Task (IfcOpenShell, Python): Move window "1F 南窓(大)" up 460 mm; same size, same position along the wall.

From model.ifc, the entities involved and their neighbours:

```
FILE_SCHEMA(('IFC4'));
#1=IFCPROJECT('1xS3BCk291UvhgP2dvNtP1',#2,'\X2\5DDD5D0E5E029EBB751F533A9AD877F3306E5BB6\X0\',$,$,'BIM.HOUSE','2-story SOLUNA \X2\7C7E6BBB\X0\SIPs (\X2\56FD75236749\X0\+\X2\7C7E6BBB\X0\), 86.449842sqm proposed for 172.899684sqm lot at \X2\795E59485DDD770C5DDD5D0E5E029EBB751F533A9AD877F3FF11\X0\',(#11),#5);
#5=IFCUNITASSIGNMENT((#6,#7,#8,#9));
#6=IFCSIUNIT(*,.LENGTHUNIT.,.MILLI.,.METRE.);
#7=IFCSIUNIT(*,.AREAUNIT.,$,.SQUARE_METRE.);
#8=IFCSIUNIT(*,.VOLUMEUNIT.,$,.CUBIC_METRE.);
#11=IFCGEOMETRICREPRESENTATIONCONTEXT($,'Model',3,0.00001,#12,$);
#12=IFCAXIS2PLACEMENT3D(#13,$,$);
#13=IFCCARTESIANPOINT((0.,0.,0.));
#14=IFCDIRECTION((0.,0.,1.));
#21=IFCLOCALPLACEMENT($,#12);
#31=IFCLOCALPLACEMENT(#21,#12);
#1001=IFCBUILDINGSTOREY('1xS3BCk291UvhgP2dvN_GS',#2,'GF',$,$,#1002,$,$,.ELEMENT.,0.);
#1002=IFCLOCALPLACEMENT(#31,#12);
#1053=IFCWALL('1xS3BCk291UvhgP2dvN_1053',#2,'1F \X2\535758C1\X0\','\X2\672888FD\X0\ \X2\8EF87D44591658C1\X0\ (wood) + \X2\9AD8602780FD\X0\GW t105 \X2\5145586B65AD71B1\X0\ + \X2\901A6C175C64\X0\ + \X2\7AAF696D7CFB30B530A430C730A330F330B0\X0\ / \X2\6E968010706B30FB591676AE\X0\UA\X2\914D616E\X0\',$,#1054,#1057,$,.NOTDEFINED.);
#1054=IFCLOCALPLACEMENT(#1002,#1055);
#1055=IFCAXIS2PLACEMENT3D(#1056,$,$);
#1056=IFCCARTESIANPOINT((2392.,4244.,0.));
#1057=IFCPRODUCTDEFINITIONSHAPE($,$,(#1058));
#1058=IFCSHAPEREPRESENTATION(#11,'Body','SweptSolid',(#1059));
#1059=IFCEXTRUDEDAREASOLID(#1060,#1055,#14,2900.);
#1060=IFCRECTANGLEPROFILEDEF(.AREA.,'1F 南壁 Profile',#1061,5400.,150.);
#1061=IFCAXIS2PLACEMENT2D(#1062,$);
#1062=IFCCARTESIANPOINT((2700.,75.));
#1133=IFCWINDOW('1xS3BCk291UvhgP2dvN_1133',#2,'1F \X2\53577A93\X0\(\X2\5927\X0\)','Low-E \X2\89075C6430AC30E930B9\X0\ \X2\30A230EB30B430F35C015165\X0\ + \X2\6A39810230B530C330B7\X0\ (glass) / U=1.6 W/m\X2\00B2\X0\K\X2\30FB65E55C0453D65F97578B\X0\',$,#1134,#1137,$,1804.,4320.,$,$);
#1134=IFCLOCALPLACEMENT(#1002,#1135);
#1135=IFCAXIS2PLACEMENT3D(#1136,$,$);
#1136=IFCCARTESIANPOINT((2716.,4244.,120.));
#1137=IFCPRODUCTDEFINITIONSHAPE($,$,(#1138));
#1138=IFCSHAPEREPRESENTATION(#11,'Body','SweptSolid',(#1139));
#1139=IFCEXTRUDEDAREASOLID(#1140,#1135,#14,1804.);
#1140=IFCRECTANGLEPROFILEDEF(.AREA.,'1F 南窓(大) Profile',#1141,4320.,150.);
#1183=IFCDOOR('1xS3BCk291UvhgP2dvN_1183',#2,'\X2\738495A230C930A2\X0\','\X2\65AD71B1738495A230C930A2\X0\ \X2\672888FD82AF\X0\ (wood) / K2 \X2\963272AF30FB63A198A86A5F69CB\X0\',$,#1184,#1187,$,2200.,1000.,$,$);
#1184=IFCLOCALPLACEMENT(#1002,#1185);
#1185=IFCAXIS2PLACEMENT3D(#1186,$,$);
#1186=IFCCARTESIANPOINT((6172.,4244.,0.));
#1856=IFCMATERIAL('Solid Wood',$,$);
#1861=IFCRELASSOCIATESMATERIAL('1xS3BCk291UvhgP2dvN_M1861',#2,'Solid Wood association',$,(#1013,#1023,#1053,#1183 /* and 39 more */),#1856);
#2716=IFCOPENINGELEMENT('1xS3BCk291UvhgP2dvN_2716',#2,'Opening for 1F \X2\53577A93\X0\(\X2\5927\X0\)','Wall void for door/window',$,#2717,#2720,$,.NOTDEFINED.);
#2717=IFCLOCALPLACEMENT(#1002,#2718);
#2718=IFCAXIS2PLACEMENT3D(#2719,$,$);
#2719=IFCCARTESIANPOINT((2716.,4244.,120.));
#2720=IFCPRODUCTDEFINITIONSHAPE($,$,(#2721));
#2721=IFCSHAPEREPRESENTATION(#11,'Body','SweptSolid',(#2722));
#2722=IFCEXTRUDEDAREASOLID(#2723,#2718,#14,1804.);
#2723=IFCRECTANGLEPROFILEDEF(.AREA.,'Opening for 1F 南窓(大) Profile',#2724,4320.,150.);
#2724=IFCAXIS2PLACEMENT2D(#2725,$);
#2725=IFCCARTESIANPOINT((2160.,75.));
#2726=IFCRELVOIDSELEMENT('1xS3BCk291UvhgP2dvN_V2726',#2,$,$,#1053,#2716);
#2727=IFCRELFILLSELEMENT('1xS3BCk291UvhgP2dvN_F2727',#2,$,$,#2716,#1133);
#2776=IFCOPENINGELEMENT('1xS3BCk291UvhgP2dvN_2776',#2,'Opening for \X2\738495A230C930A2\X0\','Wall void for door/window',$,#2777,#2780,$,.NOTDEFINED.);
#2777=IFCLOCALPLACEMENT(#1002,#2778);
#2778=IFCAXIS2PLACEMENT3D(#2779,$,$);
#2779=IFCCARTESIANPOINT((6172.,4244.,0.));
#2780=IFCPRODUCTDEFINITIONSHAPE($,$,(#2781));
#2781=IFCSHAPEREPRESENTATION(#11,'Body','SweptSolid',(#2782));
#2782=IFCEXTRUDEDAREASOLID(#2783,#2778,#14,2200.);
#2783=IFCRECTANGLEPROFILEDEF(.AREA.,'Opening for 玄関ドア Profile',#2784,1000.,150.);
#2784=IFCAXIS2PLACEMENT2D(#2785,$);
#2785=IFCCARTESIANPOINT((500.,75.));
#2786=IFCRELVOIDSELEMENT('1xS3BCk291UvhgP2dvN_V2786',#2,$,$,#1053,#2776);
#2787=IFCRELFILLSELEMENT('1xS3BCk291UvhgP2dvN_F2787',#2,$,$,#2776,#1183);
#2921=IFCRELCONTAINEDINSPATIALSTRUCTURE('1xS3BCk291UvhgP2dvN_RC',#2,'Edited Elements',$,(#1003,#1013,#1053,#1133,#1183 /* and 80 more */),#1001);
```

```python
import numpy as np
import ifcopenshell
import ifcopenshell.api.geometry
import ifcopenshell.util.placement
import ifcopenshell.util.unit

model = ifcopenshell.open("model.ifc")
unit_scale = ifcopenshell.util.unit.calculate_unit_scale(model)

window = model.by_guid("1xS3BCk291UvhgP2dvN_1133")
opening = window.FillsVoids[0].RelatingOpeningElement
dz = 460.0

shift = np.array([0.0, 0.0, dz])
# The window is not placed relative to its opening, so move both.
for product in (opening, window):
    matrix = ifcopenshell.util.placement.get_local_placement(product.ObjectPlacement)
    matrix[:3, 3] += shift
    ifcopenshell.api.geometry.edit_object_placement(model, product=product, matrix=matrix, is_si=False)

print(f"moved by {dz * unit_scale:+.3f} m")

model.write("model-out.ifc")
```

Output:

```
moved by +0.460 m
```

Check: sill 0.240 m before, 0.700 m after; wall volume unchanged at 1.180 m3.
